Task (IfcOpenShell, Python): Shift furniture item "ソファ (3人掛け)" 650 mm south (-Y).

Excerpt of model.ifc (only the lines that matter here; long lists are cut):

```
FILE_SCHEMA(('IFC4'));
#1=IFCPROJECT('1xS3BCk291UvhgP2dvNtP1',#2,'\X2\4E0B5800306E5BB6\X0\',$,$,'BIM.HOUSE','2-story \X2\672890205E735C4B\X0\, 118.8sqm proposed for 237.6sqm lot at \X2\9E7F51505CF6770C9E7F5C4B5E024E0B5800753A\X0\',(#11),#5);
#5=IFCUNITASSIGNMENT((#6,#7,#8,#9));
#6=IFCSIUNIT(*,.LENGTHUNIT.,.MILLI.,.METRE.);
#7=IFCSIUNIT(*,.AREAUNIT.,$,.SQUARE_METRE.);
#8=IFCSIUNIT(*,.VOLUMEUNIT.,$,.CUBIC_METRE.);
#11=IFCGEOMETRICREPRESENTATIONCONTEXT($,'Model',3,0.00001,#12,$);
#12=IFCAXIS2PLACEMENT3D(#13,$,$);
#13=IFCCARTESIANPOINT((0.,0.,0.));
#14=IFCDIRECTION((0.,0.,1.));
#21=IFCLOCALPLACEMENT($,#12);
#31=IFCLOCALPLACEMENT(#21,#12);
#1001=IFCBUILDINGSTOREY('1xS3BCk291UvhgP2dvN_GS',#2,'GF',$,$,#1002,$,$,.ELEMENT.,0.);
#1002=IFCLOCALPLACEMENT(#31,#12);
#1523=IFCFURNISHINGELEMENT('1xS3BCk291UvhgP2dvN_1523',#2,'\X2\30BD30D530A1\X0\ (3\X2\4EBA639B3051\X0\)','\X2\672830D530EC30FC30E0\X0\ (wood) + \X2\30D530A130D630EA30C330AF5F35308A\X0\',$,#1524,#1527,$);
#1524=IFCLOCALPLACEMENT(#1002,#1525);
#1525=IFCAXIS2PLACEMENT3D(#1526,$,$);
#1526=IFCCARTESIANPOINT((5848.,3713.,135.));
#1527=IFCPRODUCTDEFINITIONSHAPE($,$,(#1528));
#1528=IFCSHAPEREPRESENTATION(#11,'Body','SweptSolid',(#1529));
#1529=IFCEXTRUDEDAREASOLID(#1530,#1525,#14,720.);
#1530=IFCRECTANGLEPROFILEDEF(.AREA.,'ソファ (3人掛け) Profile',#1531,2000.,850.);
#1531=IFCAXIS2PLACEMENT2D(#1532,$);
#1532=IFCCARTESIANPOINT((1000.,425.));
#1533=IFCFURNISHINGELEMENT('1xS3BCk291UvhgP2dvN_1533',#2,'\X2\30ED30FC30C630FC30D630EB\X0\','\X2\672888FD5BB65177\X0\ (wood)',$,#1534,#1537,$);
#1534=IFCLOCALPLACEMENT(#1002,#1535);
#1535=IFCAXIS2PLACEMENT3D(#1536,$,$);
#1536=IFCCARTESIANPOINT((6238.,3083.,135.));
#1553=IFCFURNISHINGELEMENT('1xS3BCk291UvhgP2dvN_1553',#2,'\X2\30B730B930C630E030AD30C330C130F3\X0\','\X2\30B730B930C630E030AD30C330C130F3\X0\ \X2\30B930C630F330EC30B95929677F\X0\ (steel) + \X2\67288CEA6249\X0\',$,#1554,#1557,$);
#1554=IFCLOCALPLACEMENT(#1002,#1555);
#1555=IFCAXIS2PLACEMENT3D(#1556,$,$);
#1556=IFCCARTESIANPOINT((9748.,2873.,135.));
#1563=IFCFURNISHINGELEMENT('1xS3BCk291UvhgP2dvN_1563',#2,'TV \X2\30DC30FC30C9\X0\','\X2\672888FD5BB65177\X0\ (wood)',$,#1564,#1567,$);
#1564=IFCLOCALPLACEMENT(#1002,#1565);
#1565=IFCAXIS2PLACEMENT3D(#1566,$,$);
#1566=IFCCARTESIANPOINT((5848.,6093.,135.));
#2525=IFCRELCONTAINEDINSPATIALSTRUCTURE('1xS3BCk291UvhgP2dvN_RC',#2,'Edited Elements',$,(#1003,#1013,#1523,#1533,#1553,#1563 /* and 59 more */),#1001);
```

```python
import ifcopenshell
import ifcopenshell.api.geometry
import ifcopenshell.util.placement
import ifcopenshell.util.unit

model = ifcopenshell.open("model.ifc")
unit_scale = ifcopenshell.util.unit.calculate_unit_scale(model)

item = model.by_id(1523)
matrix = ifcopenshell.util.placement.get_local_placement(item.ObjectPlacement)
matrix[1, 3] -= 0.65 / unit_scale
ifcopenshell.api.geometry.edit_object_placement(model, product=item, matrix=matrix, is_si=False)

print(ifcopenshell.util.placement.get_local_placement(item.ObjectPlacement).round(3) + 0.0)

model.write("model_rev.ifc")
```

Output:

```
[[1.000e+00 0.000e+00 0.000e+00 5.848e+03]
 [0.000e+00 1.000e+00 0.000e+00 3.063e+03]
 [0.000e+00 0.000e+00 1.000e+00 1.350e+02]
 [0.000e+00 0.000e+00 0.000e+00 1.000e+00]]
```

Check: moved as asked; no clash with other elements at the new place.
